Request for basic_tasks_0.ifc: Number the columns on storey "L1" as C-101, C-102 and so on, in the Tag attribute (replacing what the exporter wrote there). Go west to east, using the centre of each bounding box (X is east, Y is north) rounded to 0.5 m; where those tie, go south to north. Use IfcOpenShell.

First a look at what the model holds.

```python
import ifcopenshell
import ifcopenshell.util.element
import ifcopenshell.util.placement

model = ifcopenshell.open("basic_tasks_0.ifc")
print(model.schema)
storey = next(s for s in model.by_type("IfcBuildingStorey") if s.Name == "L1")
columns = [e for e in ifcopenshell.util.element.get_decomposition(storey) if e.is_a("IfcColumn")]
for e in sorted(columns, key=lambda e: e.id()):
    origin = ifcopenshell.util.placement.get_local_placement(e.ObjectPlacement)[:3, 3]
    print(e.id(), e.Tag, e.Name, origin.round(2) + 0.0, sep=" | ")
```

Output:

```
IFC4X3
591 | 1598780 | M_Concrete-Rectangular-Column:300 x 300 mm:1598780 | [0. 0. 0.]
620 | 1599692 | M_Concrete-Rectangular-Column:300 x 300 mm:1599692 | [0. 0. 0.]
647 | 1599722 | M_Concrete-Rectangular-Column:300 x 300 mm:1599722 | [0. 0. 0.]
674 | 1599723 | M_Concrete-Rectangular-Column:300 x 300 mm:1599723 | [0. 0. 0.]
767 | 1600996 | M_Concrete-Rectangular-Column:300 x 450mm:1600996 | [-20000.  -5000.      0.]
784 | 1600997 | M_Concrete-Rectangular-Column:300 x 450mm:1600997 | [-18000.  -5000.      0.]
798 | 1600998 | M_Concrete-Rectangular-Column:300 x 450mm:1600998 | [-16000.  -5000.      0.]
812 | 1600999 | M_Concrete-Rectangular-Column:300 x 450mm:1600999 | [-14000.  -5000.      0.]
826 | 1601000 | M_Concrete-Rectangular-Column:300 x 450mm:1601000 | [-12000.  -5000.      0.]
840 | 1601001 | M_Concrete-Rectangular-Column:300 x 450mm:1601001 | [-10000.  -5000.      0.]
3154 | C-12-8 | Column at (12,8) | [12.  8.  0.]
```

```python
import ifcopenshell
import ifcopenshell.geom
import ifcopenshell.util.element
import ifcopenshell.util.shape

model = ifcopenshell.open("basic_tasks_0.ifc")
settings = ifcopenshell.geom.settings()
settings.set("use-world-coords", True)


def centre(element):
    shape = ifcopenshell.geom.create_shape(settings, element)
    return ifcopenshell.util.shape.get_bbox_centroid(shape.geometry)


storey = next(s for s in model.by_type("IfcBuildingStorey") if s.Name == "L1")
columns = [e for e in ifcopenshell.util.element.get_decomposition(storey) if e.is_a("IfcColumn")]

# Insertion points can sit at a corner or the storey origin, so sort by the geometry (in metres).
centres = {e: centre(e) for e in columns}
columns.sort(key=lambda e: (round(centres[e][0] / 0.5), centres[e][1]))

for i, e in enumerate(columns, start=1):
    number = f"C-1{i:02d}"
    e.Tag = number
    print(e.id(), number)

model.write("basic_tasks_0_rev.ifc")
```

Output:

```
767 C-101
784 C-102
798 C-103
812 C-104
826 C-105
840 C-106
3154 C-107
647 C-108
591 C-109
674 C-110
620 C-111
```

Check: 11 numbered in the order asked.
